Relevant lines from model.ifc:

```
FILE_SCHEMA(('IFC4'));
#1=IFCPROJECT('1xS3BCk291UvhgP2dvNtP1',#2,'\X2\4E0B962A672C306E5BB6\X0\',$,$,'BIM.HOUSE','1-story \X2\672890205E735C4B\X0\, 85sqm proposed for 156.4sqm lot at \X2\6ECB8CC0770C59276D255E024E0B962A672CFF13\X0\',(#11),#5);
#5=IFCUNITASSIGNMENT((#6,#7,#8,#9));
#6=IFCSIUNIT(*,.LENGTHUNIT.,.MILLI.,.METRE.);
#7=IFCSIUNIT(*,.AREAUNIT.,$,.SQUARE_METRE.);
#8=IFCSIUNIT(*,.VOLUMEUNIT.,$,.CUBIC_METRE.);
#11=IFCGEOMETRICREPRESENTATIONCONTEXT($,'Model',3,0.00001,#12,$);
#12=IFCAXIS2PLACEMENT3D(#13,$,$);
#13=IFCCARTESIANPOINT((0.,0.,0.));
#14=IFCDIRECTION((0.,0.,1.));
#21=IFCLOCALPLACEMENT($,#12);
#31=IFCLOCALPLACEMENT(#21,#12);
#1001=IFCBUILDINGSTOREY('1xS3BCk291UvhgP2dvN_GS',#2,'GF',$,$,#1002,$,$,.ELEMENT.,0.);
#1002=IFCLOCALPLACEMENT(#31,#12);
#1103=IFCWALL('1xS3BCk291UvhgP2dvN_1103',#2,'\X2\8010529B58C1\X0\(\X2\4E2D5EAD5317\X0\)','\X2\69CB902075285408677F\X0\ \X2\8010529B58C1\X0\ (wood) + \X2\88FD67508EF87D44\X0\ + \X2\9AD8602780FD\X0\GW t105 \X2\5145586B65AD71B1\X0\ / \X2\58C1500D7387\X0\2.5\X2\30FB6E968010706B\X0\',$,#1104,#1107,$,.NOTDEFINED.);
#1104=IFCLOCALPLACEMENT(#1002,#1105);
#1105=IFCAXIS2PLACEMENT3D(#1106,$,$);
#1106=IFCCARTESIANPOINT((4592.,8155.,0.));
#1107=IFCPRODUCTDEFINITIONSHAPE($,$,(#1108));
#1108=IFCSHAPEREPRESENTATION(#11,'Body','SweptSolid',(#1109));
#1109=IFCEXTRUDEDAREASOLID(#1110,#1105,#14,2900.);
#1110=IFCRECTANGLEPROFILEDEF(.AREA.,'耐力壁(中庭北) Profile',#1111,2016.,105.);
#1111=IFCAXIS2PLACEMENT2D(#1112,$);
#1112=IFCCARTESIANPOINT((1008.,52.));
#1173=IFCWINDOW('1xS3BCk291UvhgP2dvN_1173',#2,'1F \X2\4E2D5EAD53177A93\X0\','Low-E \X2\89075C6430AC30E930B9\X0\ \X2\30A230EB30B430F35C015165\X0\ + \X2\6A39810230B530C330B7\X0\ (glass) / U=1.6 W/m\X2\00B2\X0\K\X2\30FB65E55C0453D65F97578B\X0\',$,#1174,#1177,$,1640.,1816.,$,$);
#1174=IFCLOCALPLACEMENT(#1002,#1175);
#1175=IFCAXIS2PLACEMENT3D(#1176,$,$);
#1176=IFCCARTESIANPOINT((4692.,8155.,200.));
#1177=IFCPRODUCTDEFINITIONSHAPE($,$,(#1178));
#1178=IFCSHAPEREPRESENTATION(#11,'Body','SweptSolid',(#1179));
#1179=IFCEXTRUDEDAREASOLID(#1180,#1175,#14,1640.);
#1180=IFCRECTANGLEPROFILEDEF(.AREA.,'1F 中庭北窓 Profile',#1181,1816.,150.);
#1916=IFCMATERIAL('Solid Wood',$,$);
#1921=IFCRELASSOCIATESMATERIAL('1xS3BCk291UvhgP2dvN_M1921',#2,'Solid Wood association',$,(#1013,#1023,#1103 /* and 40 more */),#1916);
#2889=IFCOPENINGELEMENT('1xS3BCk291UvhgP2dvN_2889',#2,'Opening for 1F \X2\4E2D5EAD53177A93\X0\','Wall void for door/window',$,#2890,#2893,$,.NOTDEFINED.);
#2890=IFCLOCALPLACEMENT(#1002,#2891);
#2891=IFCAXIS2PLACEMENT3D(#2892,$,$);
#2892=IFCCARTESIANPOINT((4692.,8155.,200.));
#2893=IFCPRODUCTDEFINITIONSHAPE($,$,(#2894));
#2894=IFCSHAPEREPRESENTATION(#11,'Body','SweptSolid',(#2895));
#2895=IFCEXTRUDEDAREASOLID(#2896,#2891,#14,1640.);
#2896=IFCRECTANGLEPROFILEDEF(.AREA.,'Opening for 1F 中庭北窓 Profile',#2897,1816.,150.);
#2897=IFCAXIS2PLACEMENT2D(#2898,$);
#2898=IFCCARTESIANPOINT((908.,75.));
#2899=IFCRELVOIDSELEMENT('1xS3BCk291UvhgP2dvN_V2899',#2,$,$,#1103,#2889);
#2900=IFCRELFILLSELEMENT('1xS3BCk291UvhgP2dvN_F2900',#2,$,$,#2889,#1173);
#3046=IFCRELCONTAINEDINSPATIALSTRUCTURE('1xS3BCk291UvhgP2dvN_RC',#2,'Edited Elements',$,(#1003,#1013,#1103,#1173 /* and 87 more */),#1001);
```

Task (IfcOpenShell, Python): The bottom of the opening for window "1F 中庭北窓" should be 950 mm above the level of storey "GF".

```python
import numpy as np
import ifcopenshell
import ifcopenshell.api.geometry
import ifcopenshell.geom
import ifcopenshell.util.element
import ifcopenshell.util.placement
import ifcopenshell.util.shape
import ifcopenshell.util.unit

model = ifcopenshell.open("model.ifc")
unit_scale = ifcopenshell.util.unit.calculate_unit_scale(model)

window = model.by_id(1173)
opening = window.FillsVoids[0].RelatingOpeningElement
storey = ifcopenshell.util.element.get_container(window, ifc_class="IfcBuildingStorey")
level = ifcopenshell.util.placement.get_local_placement(storey.ObjectPlacement)[2, 3]

# The opening's origin need not be at the sill, so measure its lowest point.
shape = ifcopenshell.geom.create_shape(ifcopenshell.geom.settings(), opening)
bottom = ifcopenshell.util.shape.get_shape_bottom_elevation(shape, shape.geometry) / unit_scale
dz = level + 0.95 / unit_scale - bottom

shift = np.array([0.0, 0.0, dz])
# The window is not placed relative to its opening, so move both.
for product in (opening, window):
    matrix = ifcopenshell.util.placement.get_local_placement(product.ObjectPlacement)
    matrix[:3, 3] += shift
    ifcopenshell.api.geometry.edit_object_placement(model, product=product, matrix=matrix, is_si=False)

print(f"moved by {dz * unit_scale:+.3f} m")

model.write("model-out.ifc")
```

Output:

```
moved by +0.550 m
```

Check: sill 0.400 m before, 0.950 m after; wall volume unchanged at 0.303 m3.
